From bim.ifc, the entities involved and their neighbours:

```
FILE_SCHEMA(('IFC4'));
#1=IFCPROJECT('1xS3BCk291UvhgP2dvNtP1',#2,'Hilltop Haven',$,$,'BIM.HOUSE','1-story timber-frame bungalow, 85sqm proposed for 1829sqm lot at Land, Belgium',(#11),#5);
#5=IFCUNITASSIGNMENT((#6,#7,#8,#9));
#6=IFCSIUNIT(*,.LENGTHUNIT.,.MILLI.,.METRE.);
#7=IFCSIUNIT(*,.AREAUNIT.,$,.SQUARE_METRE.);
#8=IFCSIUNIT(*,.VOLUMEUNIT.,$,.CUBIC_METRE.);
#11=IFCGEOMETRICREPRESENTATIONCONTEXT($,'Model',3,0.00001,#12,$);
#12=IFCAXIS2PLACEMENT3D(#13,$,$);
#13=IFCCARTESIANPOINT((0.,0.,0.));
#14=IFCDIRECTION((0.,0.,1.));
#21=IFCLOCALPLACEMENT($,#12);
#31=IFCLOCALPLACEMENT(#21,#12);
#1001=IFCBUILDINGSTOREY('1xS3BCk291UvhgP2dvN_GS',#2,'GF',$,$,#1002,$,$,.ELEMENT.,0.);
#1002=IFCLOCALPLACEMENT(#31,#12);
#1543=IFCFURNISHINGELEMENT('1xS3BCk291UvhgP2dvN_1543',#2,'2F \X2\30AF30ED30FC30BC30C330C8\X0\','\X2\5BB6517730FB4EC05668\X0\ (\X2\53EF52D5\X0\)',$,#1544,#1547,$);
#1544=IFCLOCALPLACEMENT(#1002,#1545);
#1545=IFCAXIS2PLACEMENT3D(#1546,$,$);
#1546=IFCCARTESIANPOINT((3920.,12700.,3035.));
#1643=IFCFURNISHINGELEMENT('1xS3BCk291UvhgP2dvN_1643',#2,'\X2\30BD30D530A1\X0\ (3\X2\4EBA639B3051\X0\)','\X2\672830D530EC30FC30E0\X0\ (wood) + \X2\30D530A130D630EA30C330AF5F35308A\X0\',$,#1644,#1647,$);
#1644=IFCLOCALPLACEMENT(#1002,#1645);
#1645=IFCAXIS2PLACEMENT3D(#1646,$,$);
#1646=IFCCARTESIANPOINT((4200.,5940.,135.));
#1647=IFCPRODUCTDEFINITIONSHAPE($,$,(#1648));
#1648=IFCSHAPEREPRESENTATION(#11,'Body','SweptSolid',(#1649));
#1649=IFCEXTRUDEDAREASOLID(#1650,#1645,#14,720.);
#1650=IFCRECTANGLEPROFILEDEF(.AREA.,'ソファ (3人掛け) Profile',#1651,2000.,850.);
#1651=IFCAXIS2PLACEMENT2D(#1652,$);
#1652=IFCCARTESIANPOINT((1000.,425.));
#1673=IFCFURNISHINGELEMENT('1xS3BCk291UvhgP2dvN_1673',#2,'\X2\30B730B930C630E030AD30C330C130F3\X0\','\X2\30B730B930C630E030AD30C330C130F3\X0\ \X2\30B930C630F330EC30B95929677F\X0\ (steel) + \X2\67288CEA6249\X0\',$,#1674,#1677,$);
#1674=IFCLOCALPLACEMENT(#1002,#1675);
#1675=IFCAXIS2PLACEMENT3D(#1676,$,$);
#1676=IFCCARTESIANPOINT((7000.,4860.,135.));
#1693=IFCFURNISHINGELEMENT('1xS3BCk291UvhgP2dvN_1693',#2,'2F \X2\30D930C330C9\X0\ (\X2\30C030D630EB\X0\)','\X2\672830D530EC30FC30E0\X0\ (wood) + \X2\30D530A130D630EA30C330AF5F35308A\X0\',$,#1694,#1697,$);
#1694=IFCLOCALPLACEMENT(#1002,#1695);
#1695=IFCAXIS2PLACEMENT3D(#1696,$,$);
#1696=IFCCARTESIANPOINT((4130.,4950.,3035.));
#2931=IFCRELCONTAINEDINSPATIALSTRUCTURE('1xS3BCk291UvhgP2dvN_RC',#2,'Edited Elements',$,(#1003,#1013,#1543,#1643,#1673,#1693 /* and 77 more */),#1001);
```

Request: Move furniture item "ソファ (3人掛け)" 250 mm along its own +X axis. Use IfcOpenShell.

```python
import ifcopenshell
import ifcopenshell.api.geometry
import ifcopenshell.util.placement

model = ifcopenshell.open("bim.ifc")

item = model.by_guid("1xS3BCk291UvhgP2dvN_1643")
matrix = ifcopenshell.util.placement.get_local_placement(item.ObjectPlacement)
matrix[:3, 3] += matrix[:3, 0] * 250.0
ifcopenshell.api.geometry.edit_object_placement(model, product=item, matrix=matrix, is_si=False)

print(ifcopenshell.util.placement.get_local_placement(item.ObjectPlacement).round(3) + 0.0)

model.write("bim_updated.ifc")
```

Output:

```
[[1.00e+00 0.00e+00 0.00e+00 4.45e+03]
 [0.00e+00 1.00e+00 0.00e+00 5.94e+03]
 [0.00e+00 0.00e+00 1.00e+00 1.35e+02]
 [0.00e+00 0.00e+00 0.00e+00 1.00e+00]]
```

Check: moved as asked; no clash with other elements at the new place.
